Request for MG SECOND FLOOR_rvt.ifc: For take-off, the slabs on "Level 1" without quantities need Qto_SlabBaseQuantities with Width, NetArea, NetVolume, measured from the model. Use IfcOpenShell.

First a look at what the model holds.

```python
import ifcopenshell
import ifcopenshell.util.element
import ifcopenshell.util.unit

model = ifcopenshell.open("MG SECOND FLOOR_rvt.ifc")
print(model.schema)
for unit_type in ("LENGTHUNIT", "AREAUNIT", "VOLUMEUNIT"):
    print(unit_type, ifcopenshell.util.unit.calculate_unit_scale(model, unit_type))
storey = next(s for s in model.by_type("IfcBuildingStorey") if s.Name == "Level 1")
slabs = [e for e in ifcopenshell.util.element.get_decomposition(storey) if e.is_a("IfcSlab")]
for e in sorted(slabs, key=lambda e: e.id()):
    print(e.id(), e.is_a(), e.Name, list(ifcopenshell.util.element.get_psets(e, qtos_only=True)), sep=" | ")
```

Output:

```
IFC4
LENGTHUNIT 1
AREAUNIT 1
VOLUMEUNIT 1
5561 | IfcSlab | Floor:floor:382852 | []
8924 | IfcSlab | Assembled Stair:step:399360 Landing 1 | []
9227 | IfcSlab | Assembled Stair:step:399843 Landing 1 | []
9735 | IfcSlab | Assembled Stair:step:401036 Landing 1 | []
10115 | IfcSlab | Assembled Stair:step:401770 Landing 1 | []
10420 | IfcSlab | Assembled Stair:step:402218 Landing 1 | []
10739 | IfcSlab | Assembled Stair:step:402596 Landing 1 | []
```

```python
import ifcopenshell
import ifcopenshell.api.pset
import ifcopenshell.geom
import ifcopenshell.util.element
import ifcopenshell.util.shape
import ifcopenshell.util.unit

model = ifcopenshell.open("MG SECOND FLOOR_rvt.ifc")
unit_scale = ifcopenshell.util.unit.calculate_unit_scale(model)
area_scale = ifcopenshell.util.unit.calculate_unit_scale(model, "AREAUNIT")
volume_scale = ifcopenshell.util.unit.calculate_unit_scale(model, "VOLUMEUNIT")
settings = ifcopenshell.geom.settings()

storey = next(s for s in model.by_type("IfcBuildingStorey") if s.Name == "Level 1")
slabs = [e for e in ifcopenshell.util.element.get_decomposition(storey) if e.is_a("IfcSlab")]

for e in sorted(slabs, key=lambda e: e.id()):
    if ifcopenshell.util.element.get_psets(e, qtos_only=True, should_inherit=False):
        continue
    # Geometry comes back in metres, in the element's own axes.
    shape = ifcopenshell.geom.create_shape(settings, e)
    values = {
        "Width": ifcopenshell.util.shape.get_z(shape.geometry) / unit_scale,
        "NetArea": ifcopenshell.util.shape.get_footprint_area(shape.geometry) / area_scale,
        "NetVolume": ifcopenshell.util.shape.get_volume(shape.geometry) / volume_scale,
    }
    qto = ifcopenshell.api.pset.add_qto(model, product=e, name="Qto_SlabBaseQuantities")
    ifcopenshell.api.pset.edit_qto(model, qto=qto, properties=values)
    print(e.id(), {k: round(v, 3) for k, v in values.items()})

model.write("MG SECOND FLOOR_rvt_updated.ifc")
```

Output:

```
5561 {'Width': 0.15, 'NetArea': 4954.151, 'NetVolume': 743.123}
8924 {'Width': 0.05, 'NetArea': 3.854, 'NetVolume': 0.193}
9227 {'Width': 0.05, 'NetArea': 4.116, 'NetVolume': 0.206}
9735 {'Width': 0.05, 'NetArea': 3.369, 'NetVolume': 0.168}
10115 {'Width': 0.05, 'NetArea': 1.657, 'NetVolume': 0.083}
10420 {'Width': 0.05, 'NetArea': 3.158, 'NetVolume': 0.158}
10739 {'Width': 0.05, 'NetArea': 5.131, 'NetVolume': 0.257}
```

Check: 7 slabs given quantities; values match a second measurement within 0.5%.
